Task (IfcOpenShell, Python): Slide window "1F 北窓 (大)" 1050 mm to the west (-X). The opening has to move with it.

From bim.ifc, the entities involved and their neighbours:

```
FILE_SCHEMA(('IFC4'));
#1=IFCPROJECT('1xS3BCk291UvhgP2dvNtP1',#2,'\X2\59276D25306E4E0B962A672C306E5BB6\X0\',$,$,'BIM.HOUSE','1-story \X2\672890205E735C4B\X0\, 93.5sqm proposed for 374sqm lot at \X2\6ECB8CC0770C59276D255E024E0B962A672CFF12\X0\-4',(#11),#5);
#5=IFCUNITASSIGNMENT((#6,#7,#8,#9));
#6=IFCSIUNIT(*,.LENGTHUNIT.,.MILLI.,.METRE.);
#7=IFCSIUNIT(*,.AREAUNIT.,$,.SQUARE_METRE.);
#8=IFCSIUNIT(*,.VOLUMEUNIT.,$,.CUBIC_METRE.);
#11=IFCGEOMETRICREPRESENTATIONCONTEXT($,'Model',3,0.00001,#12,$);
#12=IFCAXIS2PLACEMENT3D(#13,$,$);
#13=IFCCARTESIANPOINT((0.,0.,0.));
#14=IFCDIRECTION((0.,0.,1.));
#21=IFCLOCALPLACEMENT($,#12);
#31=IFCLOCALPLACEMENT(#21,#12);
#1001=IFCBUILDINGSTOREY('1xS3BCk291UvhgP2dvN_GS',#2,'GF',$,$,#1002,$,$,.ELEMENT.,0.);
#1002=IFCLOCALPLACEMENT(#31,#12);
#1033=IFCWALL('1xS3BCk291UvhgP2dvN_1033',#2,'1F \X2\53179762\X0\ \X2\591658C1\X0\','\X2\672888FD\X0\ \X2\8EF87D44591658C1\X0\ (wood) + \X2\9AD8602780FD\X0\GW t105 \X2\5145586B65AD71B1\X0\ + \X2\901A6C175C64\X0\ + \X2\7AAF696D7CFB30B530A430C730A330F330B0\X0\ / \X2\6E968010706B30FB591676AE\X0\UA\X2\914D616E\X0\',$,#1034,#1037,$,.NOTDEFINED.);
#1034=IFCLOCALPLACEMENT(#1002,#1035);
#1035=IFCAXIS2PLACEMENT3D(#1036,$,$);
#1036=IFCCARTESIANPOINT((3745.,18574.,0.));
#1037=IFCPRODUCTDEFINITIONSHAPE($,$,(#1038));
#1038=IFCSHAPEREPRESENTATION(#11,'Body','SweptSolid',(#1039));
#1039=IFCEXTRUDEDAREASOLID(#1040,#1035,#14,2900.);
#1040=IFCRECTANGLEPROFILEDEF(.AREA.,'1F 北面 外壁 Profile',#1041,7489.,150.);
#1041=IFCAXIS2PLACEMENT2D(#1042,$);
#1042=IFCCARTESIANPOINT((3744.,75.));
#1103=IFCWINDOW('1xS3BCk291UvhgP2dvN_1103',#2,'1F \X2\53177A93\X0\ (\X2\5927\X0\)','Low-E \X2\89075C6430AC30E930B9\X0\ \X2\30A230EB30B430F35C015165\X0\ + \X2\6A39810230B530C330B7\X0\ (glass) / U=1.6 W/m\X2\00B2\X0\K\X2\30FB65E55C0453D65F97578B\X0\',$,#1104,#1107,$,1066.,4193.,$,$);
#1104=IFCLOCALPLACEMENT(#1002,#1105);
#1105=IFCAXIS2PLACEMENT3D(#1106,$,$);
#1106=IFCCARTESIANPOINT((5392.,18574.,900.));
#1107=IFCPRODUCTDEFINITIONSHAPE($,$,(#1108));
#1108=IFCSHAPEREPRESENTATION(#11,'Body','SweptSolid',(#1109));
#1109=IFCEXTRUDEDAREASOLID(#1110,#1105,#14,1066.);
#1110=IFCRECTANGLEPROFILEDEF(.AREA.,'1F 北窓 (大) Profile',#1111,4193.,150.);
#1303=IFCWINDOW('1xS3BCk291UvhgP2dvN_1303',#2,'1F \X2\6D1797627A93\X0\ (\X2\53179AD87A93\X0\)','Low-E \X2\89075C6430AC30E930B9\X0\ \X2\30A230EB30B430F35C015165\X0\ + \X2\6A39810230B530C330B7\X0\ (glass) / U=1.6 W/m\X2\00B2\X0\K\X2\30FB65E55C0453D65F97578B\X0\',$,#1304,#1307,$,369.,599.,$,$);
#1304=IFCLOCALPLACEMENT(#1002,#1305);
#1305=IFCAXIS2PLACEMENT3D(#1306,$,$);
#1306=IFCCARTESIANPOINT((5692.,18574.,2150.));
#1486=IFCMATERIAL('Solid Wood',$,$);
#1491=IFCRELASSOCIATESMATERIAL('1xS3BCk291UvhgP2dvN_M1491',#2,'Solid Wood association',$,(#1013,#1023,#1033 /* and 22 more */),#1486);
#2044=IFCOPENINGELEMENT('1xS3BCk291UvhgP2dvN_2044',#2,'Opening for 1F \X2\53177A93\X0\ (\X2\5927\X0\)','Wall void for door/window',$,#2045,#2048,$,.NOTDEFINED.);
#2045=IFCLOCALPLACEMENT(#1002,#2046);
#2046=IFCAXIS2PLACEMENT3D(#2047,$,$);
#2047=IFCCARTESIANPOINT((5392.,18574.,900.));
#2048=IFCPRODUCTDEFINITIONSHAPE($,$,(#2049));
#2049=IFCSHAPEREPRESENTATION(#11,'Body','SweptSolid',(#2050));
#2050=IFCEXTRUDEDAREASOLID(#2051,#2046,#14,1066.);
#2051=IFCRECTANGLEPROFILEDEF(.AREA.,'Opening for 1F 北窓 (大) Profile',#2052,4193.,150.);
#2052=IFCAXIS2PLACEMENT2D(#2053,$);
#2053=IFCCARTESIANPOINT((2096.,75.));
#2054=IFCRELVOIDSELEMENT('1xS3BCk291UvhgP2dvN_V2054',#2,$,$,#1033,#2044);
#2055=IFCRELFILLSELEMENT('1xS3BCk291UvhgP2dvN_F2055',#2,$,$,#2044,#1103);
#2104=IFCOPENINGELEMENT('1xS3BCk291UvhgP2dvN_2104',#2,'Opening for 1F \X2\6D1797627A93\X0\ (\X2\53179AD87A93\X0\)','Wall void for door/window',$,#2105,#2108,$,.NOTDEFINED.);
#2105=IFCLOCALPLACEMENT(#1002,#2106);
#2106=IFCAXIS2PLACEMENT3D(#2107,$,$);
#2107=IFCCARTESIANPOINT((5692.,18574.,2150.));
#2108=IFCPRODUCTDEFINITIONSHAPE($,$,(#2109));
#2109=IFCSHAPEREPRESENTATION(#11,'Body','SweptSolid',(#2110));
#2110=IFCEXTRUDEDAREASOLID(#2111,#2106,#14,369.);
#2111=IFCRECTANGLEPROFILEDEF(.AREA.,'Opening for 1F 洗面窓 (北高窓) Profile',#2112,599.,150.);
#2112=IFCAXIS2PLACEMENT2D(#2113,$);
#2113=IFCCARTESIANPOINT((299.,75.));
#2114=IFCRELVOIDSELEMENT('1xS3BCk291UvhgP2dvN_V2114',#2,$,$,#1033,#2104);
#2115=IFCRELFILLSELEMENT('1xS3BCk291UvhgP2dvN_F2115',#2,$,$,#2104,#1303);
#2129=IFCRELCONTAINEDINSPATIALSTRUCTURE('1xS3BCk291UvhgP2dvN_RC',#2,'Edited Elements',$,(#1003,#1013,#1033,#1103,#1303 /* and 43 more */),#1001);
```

```python
import ifcopenshell
import ifcopenshell.api.geometry
import ifcopenshell.util.placement

model = ifcopenshell.open("bim.ifc")

window = model.by_id(1103)
opening = window.FillsVoids[0].RelatingOpeningElement
wall = opening.VoidsElements[0].RelatingBuildingElement

wall_matrix = ifcopenshell.util.placement.get_local_placement(wall.ObjectPlacement)
shift = wall_matrix[:3, 0] * -1050.0
before = ifcopenshell.util.placement.get_local_placement(window.ObjectPlacement)[:3, 3].copy()

# The window is not placed relative to its opening, so move both.
for product in (opening, window):
    matrix = ifcopenshell.util.placement.get_local_placement(product.ObjectPlacement)
    matrix[:3, 3] += shift
    ifcopenshell.api.geometry.edit_object_placement(model, product=product, matrix=matrix, is_si=False)

after = ifcopenshell.util.placement.get_local_placement(window.ObjectPlacement)[:3, 3]
print("window moved by", (after - before).round(3) + 0.0)

model.write("bim_updated.ifc")
```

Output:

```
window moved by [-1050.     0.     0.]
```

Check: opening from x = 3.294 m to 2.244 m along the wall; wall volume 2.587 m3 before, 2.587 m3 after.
